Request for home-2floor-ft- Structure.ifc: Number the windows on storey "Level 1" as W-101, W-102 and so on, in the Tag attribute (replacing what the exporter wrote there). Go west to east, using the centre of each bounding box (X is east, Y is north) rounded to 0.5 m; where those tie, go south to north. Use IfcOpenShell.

First a look at what the model holds.

```python
import ifcopenshell
import ifcopenshell.util.element
import ifcopenshell.util.placement

model = ifcopenshell.open("home-2floor-ft- Structure.ifc")
print(model.schema)
storey = next(s for s in model.by_type("IfcBuildingStorey") if s.Name == "Level 1")
windows = [e for e in ifcopenshell.util.element.get_decomposition(storey) if e.is_a("IfcWindow")]
for e in sorted(windows, key=lambda e: e.id()):
    origin = ifcopenshell.util.placement.get_local_placement(e.ObjectPlacement)[:3, 3]
    print(e.id(), e.Tag, e.Name, origin.round(2) + 0.0, sep=" | ")
```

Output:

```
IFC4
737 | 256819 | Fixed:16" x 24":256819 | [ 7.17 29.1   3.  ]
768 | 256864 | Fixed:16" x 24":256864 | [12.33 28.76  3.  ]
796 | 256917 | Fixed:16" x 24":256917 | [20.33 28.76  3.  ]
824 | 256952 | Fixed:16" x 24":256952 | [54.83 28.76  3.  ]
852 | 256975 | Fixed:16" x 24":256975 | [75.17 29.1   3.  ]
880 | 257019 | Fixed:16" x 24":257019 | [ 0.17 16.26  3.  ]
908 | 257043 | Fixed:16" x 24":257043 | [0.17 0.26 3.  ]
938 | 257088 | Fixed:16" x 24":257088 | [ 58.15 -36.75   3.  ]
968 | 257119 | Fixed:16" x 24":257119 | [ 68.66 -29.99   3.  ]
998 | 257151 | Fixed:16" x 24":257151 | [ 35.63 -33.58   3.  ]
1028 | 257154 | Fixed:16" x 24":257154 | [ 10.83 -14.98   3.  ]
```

```python
import ifcopenshell
import ifcopenshell.geom
import ifcopenshell.util.element
import ifcopenshell.util.shape

model = ifcopenshell.open("home-2floor-ft- Structure.ifc")
settings = ifcopenshell.geom.settings()
settings.set("use-world-coords", True)


def centre(element):
    shape = ifcopenshell.geom.create_shape(settings, element)
    return ifcopenshell.util.shape.get_bbox_centroid(shape.geometry)


storey = next(s for s in model.by_type("IfcBuildingStorey") if s.Name == "Level 1")
windows = [e for e in ifcopenshell.util.element.get_decomposition(storey) if e.is_a("IfcWindow")]

# Insertion points can sit at a corner or the storey origin, so sort by the geometry (in metres).
centres = {e: centre(e) for e in windows}
windows.sort(key=lambda e: (round(centres[e][0] / 0.5), centres[e][1]))

for i, e in enumerate(windows, start=1):
    number = f"W-1{i:02d}"
    e.Tag = number
    print(e.id(), number)

model.write("home-2floor-ft- Structure_rev.ifc")
```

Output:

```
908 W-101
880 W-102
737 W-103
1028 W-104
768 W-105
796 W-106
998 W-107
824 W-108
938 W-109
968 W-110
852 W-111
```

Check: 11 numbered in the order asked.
